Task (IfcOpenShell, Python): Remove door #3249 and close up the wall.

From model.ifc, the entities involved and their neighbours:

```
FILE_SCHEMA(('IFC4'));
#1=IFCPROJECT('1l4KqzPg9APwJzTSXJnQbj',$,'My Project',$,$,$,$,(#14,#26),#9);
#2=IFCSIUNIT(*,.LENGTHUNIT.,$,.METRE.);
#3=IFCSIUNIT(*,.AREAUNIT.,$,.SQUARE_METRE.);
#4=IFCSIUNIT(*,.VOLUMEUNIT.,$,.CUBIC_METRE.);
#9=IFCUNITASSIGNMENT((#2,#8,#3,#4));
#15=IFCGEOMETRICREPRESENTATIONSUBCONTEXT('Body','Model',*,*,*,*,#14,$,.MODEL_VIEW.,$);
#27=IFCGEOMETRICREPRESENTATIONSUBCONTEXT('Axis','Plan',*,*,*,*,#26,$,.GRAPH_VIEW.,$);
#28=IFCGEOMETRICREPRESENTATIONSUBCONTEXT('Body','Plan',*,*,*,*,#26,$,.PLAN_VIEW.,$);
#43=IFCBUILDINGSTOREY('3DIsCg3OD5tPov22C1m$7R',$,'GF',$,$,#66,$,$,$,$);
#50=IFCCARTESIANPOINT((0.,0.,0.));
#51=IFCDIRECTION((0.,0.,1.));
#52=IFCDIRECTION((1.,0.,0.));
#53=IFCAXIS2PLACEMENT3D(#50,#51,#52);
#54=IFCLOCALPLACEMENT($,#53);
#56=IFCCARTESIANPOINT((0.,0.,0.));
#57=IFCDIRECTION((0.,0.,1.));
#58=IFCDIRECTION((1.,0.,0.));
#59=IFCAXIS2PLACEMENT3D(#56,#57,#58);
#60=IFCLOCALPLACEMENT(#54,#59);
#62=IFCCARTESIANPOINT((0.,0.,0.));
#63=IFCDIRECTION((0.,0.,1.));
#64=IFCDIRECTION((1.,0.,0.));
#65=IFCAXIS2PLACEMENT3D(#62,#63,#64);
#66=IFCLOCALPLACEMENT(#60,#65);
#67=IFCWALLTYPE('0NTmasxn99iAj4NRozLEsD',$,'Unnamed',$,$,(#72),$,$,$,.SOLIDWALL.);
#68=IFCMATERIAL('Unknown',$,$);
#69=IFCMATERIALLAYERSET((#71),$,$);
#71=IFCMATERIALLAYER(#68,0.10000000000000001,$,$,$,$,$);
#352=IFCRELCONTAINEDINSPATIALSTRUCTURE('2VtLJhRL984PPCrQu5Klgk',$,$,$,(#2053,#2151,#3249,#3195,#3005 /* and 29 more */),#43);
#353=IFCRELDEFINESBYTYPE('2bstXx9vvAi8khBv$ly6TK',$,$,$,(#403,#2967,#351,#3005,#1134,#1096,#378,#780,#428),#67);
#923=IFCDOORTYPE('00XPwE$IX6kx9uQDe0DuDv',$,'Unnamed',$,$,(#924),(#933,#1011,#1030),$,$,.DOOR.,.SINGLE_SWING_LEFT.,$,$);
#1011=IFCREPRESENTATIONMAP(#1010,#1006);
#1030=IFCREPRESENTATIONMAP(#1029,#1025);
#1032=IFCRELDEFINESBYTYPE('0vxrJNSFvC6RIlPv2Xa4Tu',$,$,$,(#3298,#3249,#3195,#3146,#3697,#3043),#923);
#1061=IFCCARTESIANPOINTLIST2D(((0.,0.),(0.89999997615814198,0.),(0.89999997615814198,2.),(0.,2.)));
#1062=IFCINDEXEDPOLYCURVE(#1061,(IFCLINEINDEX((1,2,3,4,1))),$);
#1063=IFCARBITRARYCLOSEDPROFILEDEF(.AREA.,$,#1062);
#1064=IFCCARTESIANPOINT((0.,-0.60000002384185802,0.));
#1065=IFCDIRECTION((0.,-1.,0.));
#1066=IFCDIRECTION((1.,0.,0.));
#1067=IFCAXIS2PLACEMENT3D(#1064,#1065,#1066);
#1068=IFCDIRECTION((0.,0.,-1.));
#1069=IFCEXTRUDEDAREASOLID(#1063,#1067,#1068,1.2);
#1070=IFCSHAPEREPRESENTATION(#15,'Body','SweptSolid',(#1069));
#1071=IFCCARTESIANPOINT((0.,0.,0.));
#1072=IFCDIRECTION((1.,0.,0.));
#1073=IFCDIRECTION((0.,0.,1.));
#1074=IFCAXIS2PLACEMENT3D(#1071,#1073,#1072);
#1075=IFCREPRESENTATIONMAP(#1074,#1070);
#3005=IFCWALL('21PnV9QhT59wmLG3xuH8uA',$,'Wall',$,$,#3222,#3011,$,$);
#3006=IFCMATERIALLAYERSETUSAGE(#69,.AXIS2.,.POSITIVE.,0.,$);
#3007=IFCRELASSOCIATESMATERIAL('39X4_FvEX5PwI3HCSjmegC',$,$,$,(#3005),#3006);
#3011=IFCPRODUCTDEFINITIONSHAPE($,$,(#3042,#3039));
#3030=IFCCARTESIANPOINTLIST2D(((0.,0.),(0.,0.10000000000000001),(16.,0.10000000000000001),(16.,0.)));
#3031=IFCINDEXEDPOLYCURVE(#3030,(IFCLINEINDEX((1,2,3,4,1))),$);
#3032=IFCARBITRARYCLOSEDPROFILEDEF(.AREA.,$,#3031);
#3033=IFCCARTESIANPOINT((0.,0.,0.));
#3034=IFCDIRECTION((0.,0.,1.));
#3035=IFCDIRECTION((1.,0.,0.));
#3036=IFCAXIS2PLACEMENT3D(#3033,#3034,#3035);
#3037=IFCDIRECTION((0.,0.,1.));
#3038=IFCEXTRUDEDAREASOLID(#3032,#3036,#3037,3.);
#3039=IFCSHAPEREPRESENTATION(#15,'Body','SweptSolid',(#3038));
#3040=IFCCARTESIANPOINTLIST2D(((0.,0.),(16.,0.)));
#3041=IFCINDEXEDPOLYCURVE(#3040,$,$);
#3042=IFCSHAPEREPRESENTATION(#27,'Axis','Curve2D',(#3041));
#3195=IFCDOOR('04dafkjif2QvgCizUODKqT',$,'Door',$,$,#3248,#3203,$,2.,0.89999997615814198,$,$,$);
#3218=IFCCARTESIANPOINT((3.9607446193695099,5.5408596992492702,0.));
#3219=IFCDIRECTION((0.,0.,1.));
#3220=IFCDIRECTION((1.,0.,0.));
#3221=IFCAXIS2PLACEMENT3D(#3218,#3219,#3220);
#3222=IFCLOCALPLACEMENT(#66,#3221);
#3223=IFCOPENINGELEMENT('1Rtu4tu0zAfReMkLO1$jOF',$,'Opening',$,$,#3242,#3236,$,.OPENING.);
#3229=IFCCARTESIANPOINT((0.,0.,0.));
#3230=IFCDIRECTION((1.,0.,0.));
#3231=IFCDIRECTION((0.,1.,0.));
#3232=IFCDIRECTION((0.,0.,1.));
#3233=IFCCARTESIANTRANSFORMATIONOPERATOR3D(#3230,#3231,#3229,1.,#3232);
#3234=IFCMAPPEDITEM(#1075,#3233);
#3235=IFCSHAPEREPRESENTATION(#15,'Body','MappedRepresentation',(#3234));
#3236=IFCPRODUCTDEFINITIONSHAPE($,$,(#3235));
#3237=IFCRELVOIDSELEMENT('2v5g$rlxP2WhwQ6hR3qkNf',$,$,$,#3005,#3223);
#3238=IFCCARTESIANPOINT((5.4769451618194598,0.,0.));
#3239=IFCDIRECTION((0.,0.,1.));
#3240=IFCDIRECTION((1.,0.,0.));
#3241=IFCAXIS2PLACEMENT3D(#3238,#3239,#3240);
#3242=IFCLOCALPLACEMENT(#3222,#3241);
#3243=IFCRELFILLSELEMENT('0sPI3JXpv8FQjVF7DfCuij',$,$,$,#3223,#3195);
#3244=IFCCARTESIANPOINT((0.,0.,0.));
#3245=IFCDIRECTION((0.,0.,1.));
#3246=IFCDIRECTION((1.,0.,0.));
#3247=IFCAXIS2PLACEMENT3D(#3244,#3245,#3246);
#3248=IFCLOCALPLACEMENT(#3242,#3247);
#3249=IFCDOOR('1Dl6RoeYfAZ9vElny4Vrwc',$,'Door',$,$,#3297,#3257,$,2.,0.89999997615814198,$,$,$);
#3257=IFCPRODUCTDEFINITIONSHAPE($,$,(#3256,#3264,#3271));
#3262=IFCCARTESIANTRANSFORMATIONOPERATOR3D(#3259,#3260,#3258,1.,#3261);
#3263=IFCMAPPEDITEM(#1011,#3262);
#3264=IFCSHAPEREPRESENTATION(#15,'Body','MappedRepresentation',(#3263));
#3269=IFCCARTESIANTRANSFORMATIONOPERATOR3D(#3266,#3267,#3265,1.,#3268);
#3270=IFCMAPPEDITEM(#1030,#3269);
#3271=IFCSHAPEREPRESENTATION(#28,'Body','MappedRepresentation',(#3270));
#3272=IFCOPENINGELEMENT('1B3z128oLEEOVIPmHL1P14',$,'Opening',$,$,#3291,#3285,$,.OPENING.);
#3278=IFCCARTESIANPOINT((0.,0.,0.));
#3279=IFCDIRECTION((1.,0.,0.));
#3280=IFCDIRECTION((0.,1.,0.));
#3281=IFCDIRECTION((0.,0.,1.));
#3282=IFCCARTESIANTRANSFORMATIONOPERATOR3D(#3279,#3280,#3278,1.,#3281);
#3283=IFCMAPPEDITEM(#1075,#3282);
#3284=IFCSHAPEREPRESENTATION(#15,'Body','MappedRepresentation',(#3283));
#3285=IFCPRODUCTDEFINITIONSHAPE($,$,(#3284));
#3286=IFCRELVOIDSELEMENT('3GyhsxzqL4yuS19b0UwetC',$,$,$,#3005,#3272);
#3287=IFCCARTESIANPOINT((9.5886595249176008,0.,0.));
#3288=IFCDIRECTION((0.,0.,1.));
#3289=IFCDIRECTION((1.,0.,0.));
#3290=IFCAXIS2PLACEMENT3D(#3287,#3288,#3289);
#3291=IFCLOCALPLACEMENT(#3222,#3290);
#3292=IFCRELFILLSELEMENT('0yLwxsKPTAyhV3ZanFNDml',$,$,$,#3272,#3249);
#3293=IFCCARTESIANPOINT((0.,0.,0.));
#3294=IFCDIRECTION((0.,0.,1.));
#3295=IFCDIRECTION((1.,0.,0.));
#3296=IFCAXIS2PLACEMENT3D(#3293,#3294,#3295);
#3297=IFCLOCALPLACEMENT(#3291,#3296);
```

```python
import ifcopenshell
import ifcopenshell.api.feature
import ifcopenshell.api.root
import ifcopenshell.geom
import ifcopenshell.util.shape

model = ifcopenshell.open("model.ifc")
settings = ifcopenshell.geom.settings()


def volume(element):
    """Net volume in cubic metres, openings subtracted."""
    shape = ifcopenshell.geom.create_shape(settings, element)
    return ifcopenshell.util.shape.get_volume(shape.geometry)


door = model.by_guid("1Dl6RoeYfAZ9vElny4Vrwc")
opening = door.FillsVoids[0].RelatingOpeningElement
wall = opening.VoidsElements[0].RelatingBuildingElement
before = volume(wall)

ifcopenshell.api.root.remove_product(model, product=door)
ifcopenshell.api.feature.remove_feature(model, feature=opening)

after = volume(wall)

print(f"wall volume {before:.3f} -> {after:.3f} m3")

model.write("model_edited.ifc")
```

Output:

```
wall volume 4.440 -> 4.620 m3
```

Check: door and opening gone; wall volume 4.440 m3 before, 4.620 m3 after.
